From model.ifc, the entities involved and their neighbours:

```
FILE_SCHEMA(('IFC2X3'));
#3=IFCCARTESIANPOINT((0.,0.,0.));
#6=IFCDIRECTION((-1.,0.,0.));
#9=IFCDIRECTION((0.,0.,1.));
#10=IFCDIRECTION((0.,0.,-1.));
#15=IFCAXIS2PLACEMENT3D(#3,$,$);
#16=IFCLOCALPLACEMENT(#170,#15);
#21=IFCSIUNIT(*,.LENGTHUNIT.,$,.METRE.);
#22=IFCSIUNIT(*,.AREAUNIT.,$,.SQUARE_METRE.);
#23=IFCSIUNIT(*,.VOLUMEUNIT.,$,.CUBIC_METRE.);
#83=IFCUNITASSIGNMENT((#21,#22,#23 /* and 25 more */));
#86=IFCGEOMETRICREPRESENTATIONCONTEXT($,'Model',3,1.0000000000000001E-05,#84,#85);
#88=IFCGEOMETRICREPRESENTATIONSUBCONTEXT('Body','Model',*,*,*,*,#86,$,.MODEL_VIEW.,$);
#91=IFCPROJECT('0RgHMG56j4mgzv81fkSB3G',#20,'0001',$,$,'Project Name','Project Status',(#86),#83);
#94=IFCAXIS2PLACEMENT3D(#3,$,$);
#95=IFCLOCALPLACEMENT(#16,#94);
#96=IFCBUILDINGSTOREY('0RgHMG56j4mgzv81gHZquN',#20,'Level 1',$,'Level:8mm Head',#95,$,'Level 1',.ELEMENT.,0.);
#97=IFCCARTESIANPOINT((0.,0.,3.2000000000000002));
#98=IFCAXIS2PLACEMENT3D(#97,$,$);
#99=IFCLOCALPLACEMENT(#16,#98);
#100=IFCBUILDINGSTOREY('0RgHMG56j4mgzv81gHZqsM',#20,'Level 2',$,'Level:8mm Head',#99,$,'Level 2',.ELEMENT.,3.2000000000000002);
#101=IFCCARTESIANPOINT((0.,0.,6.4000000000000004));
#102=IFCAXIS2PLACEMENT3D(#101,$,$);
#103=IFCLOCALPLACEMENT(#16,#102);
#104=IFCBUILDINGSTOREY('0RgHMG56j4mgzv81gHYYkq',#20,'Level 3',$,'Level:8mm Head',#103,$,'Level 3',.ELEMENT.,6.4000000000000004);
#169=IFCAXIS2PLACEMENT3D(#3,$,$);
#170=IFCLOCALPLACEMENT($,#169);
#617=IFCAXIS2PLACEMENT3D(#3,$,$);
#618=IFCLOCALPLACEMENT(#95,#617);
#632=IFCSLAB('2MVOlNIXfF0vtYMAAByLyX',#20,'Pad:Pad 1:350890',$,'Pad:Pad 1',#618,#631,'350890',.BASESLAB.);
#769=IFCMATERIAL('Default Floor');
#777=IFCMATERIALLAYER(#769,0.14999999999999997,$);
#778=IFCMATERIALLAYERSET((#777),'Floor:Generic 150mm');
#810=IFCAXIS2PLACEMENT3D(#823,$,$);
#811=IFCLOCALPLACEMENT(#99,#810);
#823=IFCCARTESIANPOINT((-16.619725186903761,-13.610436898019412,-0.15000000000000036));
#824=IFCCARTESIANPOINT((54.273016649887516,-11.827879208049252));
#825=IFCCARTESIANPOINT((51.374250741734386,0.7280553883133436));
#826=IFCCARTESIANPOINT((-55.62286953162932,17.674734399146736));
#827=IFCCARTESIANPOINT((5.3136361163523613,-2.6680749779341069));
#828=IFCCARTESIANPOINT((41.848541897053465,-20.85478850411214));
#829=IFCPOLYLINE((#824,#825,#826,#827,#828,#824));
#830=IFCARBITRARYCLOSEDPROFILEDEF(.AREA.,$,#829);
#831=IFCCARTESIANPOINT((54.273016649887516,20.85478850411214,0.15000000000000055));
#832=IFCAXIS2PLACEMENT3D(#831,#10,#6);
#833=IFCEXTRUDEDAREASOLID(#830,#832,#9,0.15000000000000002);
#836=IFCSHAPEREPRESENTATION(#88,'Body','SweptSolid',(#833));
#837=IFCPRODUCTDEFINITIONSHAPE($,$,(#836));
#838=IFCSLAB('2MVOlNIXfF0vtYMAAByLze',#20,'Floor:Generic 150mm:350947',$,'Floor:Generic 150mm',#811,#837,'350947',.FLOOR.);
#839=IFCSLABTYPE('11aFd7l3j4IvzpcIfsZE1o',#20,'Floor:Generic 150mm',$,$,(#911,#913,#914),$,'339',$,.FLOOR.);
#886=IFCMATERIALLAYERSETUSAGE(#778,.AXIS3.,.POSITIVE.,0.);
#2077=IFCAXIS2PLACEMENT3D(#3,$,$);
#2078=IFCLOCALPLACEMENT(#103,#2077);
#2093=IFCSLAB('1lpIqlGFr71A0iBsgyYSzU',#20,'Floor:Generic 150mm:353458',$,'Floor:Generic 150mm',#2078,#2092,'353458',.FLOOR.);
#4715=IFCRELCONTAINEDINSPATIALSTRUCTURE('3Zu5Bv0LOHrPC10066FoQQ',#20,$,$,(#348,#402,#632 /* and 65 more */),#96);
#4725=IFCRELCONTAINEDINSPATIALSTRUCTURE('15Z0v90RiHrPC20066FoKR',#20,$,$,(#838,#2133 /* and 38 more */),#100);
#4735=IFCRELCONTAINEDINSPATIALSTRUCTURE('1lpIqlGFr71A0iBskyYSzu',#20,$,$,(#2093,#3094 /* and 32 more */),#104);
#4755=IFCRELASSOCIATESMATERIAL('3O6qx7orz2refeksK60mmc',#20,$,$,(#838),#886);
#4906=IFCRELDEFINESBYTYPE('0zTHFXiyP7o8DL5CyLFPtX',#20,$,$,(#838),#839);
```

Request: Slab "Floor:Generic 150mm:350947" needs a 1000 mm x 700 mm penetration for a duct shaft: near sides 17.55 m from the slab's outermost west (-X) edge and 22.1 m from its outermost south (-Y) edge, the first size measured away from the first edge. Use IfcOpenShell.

```python
import numpy as np
import ifcopenshell
import ifcopenshell.api.feature
import ifcopenshell.api.geometry
import ifcopenshell.api.root
import ifcopenshell.geom
import ifcopenshell.util.placement
import ifcopenshell.util.representation
import ifcopenshell.util.shape
import ifcopenshell.util.unit

model = ifcopenshell.open("model.ifc")
unit_scale = ifcopenshell.util.unit.calculate_unit_scale(model)
settings = ifcopenshell.geom.settings()


def volume(element):
    """Net volume in cubic metres, openings subtracted."""
    shape = ifcopenshell.geom.create_shape(settings, element)
    return ifcopenshell.util.shape.get_volume(shape.geometry)


slab = model.by_id(838)
before = volume(slab)

# Extent in the slab's own axes, in metres. The edges named are its -X and -Y sides.
slab_shape = ifcopenshell.geom.create_shape(settings, slab)
vertices = ifcopenshell.util.shape.get_vertices(slab_shape.geometry)
x_min, y_min, bottom = vertices.min(axis=0)
top = vertices[:, 2].max()

opening = ifcopenshell.api.root.create_entity(model, ifc_class="IfcOpeningElement", name="Duct shaft opening")
context = ifcopenshell.util.representation.get_context(model, "Model", "Body", "MODEL_VIEW")
width, depth = 1, 0.7
outline = [(0.0, 0.0), (width, 0.0), (width, depth), (0.0, depth), (0.0, 0.0)]
# Overshoot both faces by 50 mm so the cut is clean.
shape = ifcopenshell.api.geometry.add_slab_representation(
    model, context=context, depth=top - bottom + 0.1, polyline=outline
)
ifcopenshell.api.geometry.assign_representation(model, product=opening, representation=shape)

matrix = ifcopenshell.util.placement.get_local_placement(slab.ObjectPlacement)
matrix[:, 3] = matrix @ np.append(np.array([x_min + 17.55, y_min + 22.1, bottom - 0.05]) / unit_scale, 1.0)
ifcopenshell.api.geometry.edit_object_placement(model, product=opening, matrix=matrix, is_si=False)
ifcopenshell.api.feature.add_feature(model, feature=opening, element=slab)

after = volume(slab)

print(f"slab volume {before:.3f} -> {after:.3f} m3")

model.write("model_rev.ifc")
```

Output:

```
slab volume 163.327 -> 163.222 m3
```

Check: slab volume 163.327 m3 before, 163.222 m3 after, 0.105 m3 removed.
